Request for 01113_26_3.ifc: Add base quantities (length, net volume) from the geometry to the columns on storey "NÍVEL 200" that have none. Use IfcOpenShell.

First a look at what the model holds.

```python
import ifcopenshell
import ifcopenshell.util.element
import ifcopenshell.util.unit

model = ifcopenshell.open("01113_26_3.ifc")
print(model.schema)
for unit_type in ("LENGTHUNIT", "AREAUNIT", "VOLUMEUNIT"):
    print(unit_type, ifcopenshell.util.unit.calculate_unit_scale(model, unit_type))
storey = next(s for s in model.by_type("IfcBuildingStorey") if s.Name == "NÍVEL 200")
columns = [e for e in ifcopenshell.util.element.get_decomposition(storey) if e.is_a("IfcColumn")]
for e in sorted(columns, key=lambda e: e.id()):
    print(e.id(), e.is_a(), e.Name, list(ifcopenshell.util.element.get_psets(e, qtos_only=True)), sep=" | ")
```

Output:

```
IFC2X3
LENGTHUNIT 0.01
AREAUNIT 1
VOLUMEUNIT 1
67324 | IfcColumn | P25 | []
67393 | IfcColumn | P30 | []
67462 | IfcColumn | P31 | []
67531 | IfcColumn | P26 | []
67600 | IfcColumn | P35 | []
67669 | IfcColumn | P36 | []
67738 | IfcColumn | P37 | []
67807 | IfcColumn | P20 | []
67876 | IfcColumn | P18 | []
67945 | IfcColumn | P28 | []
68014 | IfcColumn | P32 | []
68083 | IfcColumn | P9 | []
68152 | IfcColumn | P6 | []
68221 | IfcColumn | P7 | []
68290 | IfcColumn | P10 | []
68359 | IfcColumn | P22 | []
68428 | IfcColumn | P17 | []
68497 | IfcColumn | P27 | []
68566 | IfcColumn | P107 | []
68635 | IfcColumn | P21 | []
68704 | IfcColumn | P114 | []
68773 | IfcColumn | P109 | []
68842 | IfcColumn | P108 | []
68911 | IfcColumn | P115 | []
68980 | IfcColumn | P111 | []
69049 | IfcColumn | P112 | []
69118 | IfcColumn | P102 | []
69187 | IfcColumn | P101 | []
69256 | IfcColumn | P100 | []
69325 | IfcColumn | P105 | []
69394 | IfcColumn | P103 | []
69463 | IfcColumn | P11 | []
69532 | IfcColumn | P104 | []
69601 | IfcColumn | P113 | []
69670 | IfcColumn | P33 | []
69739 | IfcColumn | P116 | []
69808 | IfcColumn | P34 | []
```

```python
import ifcopenshell
import ifcopenshell.api.pset
import ifcopenshell.geom
import ifcopenshell.util.element
import ifcopenshell.util.shape
import ifcopenshell.util.unit

model = ifcopenshell.open("01113_26_3.ifc")
unit_scale = ifcopenshell.util.unit.calculate_unit_scale(model)
volume_scale = ifcopenshell.util.unit.calculate_unit_scale(model, "VOLUMEUNIT")
settings = ifcopenshell.geom.settings()

storey = next(s for s in model.by_type("IfcBuildingStorey") if s.Name == "NÍVEL 200")
columns = [e for e in ifcopenshell.util.element.get_decomposition(storey) if e.is_a("IfcColumn")]

for e in sorted(columns, key=lambda e: e.id()):
    if ifcopenshell.util.element.get_psets(e, qtos_only=True, should_inherit=False):
        continue
    # Geometry comes back in metres, in the element's own axes.
    shape = ifcopenshell.geom.create_shape(settings, e)
    values = {
        "Length": ifcopenshell.util.shape.get_z(shape.geometry) / unit_scale,
        "NetVolume": ifcopenshell.util.shape.get_volume(shape.geometry) / volume_scale,
    }
    qto = ifcopenshell.api.pset.add_qto(model, product=e, name="BaseQuantities")
    ifcopenshell.api.pset.edit_qto(model, qto=qto, properties=values)
    print(e.id(), {k: round(v, 3) for k, v in values.items()})

model.write("01113_26_3-out.ifc")
```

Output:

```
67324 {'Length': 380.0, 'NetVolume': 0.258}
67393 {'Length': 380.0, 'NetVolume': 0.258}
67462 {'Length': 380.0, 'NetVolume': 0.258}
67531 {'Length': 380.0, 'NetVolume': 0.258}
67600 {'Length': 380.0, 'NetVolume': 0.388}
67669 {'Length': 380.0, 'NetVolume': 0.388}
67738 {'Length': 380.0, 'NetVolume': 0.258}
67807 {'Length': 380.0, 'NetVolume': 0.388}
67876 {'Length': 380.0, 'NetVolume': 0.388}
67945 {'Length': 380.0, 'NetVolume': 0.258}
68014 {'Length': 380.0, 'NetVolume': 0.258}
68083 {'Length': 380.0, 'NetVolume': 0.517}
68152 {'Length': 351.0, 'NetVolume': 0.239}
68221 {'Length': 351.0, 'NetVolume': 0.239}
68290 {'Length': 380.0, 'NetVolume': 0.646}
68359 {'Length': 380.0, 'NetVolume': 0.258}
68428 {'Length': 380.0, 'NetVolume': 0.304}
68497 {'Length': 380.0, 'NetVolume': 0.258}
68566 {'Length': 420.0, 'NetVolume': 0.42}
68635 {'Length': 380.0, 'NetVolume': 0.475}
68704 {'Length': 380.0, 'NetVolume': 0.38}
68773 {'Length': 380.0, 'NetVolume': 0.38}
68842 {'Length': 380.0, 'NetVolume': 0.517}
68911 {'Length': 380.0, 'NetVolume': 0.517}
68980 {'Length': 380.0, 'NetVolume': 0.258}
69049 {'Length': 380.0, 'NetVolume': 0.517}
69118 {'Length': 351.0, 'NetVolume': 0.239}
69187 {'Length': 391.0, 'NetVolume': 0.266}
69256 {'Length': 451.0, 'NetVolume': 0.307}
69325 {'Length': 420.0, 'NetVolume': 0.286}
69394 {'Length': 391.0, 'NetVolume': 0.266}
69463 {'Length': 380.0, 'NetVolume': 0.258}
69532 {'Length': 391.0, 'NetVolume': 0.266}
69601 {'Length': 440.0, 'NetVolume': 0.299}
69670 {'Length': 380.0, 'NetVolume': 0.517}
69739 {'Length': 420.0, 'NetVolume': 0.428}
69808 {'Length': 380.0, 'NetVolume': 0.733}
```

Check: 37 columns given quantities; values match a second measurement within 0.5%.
